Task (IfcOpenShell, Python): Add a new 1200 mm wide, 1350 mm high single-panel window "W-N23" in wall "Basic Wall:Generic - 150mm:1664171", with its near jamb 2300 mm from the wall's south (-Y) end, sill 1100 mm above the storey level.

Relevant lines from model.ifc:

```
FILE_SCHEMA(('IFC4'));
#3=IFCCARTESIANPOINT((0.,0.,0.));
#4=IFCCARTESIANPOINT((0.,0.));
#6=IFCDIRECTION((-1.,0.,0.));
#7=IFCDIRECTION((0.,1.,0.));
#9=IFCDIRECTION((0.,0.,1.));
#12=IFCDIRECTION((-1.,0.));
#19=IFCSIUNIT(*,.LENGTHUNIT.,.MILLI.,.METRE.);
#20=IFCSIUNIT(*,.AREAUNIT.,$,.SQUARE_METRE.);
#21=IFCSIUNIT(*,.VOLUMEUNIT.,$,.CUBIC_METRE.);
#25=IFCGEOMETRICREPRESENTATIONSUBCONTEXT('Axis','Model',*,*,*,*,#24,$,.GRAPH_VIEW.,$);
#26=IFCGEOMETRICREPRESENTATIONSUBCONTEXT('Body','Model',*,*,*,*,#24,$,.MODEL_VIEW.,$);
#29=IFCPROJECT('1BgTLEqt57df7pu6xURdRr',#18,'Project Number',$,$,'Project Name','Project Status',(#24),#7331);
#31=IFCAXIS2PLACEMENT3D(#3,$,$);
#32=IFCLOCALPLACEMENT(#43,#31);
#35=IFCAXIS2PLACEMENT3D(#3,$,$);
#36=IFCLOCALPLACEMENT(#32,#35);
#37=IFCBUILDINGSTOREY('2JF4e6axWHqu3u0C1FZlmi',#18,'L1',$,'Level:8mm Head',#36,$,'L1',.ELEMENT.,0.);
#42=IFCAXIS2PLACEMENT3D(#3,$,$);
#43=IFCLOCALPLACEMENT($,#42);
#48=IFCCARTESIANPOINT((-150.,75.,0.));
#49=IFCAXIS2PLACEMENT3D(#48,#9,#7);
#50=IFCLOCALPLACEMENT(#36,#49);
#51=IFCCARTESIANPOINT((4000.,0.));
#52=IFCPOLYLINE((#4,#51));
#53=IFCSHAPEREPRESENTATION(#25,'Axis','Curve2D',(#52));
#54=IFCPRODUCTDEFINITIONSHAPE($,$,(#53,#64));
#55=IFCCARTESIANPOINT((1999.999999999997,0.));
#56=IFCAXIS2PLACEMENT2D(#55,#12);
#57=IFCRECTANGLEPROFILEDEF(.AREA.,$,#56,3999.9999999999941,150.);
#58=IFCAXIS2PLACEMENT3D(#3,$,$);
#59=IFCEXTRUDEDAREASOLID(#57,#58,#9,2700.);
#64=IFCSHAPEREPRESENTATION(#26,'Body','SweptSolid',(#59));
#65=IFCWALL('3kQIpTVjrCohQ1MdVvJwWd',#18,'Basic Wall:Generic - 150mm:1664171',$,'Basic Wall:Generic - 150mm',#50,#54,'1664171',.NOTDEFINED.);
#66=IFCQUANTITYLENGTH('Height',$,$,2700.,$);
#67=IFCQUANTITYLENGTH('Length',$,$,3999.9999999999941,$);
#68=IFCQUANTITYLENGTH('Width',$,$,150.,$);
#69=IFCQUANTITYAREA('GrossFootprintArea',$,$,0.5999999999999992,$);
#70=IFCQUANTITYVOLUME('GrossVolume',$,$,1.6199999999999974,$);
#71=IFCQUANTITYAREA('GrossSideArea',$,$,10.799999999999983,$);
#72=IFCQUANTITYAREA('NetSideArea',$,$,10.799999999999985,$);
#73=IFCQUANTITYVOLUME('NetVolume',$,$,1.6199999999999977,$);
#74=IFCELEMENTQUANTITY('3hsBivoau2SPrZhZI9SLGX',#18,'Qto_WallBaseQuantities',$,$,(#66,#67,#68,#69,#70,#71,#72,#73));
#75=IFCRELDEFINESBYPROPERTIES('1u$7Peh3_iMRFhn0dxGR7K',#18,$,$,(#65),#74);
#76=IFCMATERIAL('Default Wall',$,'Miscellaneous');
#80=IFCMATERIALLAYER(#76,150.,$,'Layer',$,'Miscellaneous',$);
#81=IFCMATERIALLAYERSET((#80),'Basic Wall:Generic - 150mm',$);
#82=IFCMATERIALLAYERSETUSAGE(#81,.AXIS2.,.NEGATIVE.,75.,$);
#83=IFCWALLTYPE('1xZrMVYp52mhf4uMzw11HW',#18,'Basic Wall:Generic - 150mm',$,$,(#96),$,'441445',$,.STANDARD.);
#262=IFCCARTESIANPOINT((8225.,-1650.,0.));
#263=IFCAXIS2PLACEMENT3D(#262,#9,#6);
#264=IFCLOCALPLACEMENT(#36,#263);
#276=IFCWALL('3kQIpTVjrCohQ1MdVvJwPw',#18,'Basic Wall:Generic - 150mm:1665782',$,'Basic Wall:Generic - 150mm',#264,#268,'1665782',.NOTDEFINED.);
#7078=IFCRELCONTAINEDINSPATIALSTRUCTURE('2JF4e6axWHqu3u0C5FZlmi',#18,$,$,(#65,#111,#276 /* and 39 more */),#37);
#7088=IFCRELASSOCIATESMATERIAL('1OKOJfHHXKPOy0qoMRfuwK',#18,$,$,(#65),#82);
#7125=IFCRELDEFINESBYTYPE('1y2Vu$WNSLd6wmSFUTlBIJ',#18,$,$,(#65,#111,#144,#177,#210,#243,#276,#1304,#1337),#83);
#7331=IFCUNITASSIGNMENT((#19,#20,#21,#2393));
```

```python
import numpy as np
import ifcopenshell
import ifcopenshell.api.feature
import ifcopenshell.api.geometry
import ifcopenshell.api.pset
import ifcopenshell.api.root
import ifcopenshell.api.spatial
import ifcopenshell.geom
import ifcopenshell.util.element
import ifcopenshell.util.placement
import ifcopenshell.util.representation
import ifcopenshell.util.shape
import ifcopenshell.util.unit

model = ifcopenshell.open("model.ifc")
unit_scale = ifcopenshell.util.unit.calculate_unit_scale(model)
area_scale = ifcopenshell.util.unit.calculate_unit_scale(model, "AREAUNIT")
volume_scale = ifcopenshell.util.unit.calculate_unit_scale(model, "VOLUMEUNIT")
settings = ifcopenshell.geom.settings()


def volume(element):
    """Net volume in cubic metres, openings subtracted."""
    shape = ifcopenshell.geom.create_shape(settings, element)
    return ifcopenshell.util.shape.get_volume(shape.geometry)


wall = model.by_guid("3kQIpTVjrCohQ1MdVvJwWd")
storey = ifcopenshell.util.element.get_container(wall, ifc_class="IfcBuildingStorey")
context = ifcopenshell.util.representation.get_context(model, "Model", "Body", "MODEL_VIEW")
before = volume(wall)

width, height, from_end, sill = 1.2, 1.35, 2.3, 1.1  # metres

# The wall runs along its own X axis, and the end named is its -X end.
wall_shape = ifcopenshell.geom.create_shape(settings, wall)
x, y, z = ifcopenshell.util.shape.get_vertices(wall_shape.geometry).T
start = x.min() + from_end
face, thickness = float(y.min()), float(y.max() - y.min())
wall_matrix = ifcopenshell.util.placement.get_local_placement(wall.ObjectPlacement)
level = ifcopenshell.util.placement.get_local_placement(storey.ObjectPlacement)[2, 3]


def in_wall(x, y):
    """Placement at x, y metres in the wall's axes, at sill height."""
    matrix = wall_matrix.copy()
    matrix[:, 3] = wall_matrix @ np.array([x / unit_scale, y / unit_scale, 0.0, 1.0])
    matrix[2, 3] = level + sill / unit_scale
    return matrix


# Opening: a box that overshoots both wall faces by 50 mm.
opening = ifcopenshell.api.root.create_entity(model, ifc_class="IfcOpeningElement", predefined_type="OPENING")
box = ifcopenshell.api.geometry.add_wall_representation(
    model, context=context, length=width, height=height, thickness=thickness + 0.1
)
ifcopenshell.api.geometry.assign_representation(model, product=opening, representation=box)
ifcopenshell.api.geometry.edit_object_placement(model, product=opening, matrix=in_wall(start, face - 0.05), is_si=False)
ifcopenshell.api.feature.add_feature(model, feature=opening, element=wall)

window = ifcopenshell.api.root.create_entity(model, ifc_class="IfcWindow", name="W-N23", predefined_type="WINDOW")
window.OverallWidth, window.OverallHeight = width / unit_scale, height / unit_scale
window.PartitioningType = "SINGLE_PANEL"
body = ifcopenshell.api.geometry.add_window_representation(
    model,
    context=context,
    overall_width=window.OverallWidth,
    overall_height=window.OverallHeight,
    partition_type="SINGLE_PANEL",
)
ifcopenshell.api.geometry.assign_representation(model, product=window, representation=body)
ifcopenshell.api.spatial.assign_container(model, products=[window], relating_structure=storey)
ifcopenshell.api.feature.add_filling(model, opening=opening, element=window)

# Centre the window in the wall's thickness.
ifcopenshell.api.geometry.edit_object_placement(model, product=window, matrix=in_wall(start, face), is_si=False)
window_shape = ifcopenshell.geom.create_shape(settings, window)
depth = ifcopenshell.util.shape.get_vertices(window_shape.geometry)[:, 1]
offset = face + thickness / 2 - (depth.min() + depth.max()) / 2
ifcopenshell.api.geometry.edit_object_placement(model, product=window, matrix=in_wall(start, offset), is_si=False)

after = volume(wall)

# Update the wall's stored quantities.
qto = model.by_id(ifcopenshell.util.element.get_pset(wall, "Qto_WallBaseQuantities", should_inherit=False)["id"])
ifcopenshell.api.pset.edit_qto(model, qto=qto, properties={
    "NetSideArea": after / thickness / area_scale,
    "NetVolume": after / volume_scale,
})

print(f"wall volume {before:.3f} -> {after:.3f} m3")

model.write("model_updated.ifc")
```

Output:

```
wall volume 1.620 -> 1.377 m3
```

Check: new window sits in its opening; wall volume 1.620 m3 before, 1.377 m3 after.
